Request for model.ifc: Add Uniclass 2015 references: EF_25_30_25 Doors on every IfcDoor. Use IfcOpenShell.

First a look at what the model holds.

```python
import ifcopenshell

model = ifcopenshell.open("model.ifc")
print(model.schema)
print("classifications:", [c.Name for c in model.by_type("IfcClassification")])
for ifc_class in ("IfcDoor", "IfcRoof", "IfcStair", "IfcWall", "IfcWindow"):
    print(ifc_class, len(model.by_type(ifc_class)))
```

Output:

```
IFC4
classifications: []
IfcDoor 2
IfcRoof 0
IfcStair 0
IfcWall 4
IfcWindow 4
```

```python
import ifcopenshell
import ifcopenshell.api.classification

model = ifcopenshell.open("model.ifc")

system = ifcopenshell.api.classification.add_classification(model, classification="Uniclass 2015")

codes = {
    "IfcDoor": ("EF_25_30_25", "Doors"),
}
for ifc_class, (code, name) in codes.items():
    products = model.by_type(ifc_class)
    ifcopenshell.api.classification.add_reference(
        model, products=products, classification=system, identification=code, name=name
    )
    print(code, len(products))

model.write("model_rev.ifc")
```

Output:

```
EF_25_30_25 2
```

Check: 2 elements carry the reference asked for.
